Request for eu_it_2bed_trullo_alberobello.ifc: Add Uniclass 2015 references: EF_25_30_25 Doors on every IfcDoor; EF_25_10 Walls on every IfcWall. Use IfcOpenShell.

First a look at what the model holds.

```python
import ifcopenshell

model = ifcopenshell.open("eu_it_2bed_trullo_alberobello.ifc")
print(model.schema)
print("classifications:", [c.Name for c in model.by_type("IfcClassification")])
for ifc_class in ("IfcDoor", "IfcRoof", "IfcStair", "IfcWall", "IfcWindow"):
    print(ifc_class, len(model.by_type(ifc_class)))
```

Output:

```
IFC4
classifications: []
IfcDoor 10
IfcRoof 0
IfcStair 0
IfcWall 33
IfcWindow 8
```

```python
import ifcopenshell
import ifcopenshell.api.classification

model = ifcopenshell.open("eu_it_2bed_trullo_alberobello.ifc")

system = ifcopenshell.api.classification.add_classification(model, classification="Uniclass 2015")

codes = {
    "IfcDoor": ("EF_25_30_25", "Doors"),
    "IfcWall": ("EF_25_10", "Walls"),
}
for ifc_class, (code, name) in codes.items():
    products = model.by_type(ifc_class)
    ifcopenshell.api.classification.add_reference(
        model, products=products, classification=system, identification=code, name=name
    )
    print(code, len(products))

model.write("eu_it_2bed_trullo_alberobello_rev.ifc")
```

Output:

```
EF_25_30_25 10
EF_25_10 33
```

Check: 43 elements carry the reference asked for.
